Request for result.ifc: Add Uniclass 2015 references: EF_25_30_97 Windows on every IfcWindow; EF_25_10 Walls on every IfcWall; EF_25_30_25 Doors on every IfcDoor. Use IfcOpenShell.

First a look at what the model holds.

```python
import ifcopenshell

model = ifcopenshell.open("result.ifc")
print(model.schema)
print("classifications:", [c.Name for c in model.by_type("IfcClassification")])
for ifc_class in ("IfcDoor", "IfcRoof", "IfcStair", "IfcWall", "IfcWindow"):
    print(ifc_class, len(model.by_type(ifc_class)))
```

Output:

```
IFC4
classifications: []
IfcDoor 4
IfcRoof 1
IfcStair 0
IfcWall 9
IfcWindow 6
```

```python
import ifcopenshell
import ifcopenshell.api.classification

model = ifcopenshell.open("result.ifc")

system = ifcopenshell.api.classification.add_classification(model, classification="Uniclass 2015")

codes = {
    "IfcWindow": ("EF_25_30_97", "Windows"),
    "IfcWall": ("EF_25_10", "Walls"),
    "IfcDoor": ("EF_25_30_25", "Doors"),
}
for ifc_class, (code, name) in codes.items():
    products = model.by_type(ifc_class)
    ifcopenshell.api.classification.add_reference(
        model, products=products, classification=system, identification=code, name=name
    )
    print(code, len(products))

model.write("result_edited.ifc")
```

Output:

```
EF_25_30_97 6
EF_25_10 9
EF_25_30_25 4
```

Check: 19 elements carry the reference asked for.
